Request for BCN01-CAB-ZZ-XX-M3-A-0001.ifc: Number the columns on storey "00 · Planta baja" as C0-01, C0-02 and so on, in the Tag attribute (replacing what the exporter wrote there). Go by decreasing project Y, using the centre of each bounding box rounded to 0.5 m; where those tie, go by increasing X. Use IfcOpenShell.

First a look at what the model holds.

```python
import ifcopenshell
import ifcopenshell.util.element
import ifcopenshell.util.placement

model = ifcopenshell.open("BCN01-CAB-ZZ-XX-M3-A-0001.ifc")
print(model.schema)
storey = next(s for s in model.by_type("IfcBuildingStorey") if s.Name == "00 · Planta baja")
columns = [e for e in ifcopenshell.util.element.get_decomposition(storey) if e.is_a("IfcColumn")]
for e in sorted(columns, key=lambda e: e.id()):
    origin = ifcopenshell.util.placement.get_local_placement(e.ObjectPlacement)[:3, 3]
    print(e.id(), e.Tag, e.Name, origin.round(2) + 0.0, sep=" | ")
```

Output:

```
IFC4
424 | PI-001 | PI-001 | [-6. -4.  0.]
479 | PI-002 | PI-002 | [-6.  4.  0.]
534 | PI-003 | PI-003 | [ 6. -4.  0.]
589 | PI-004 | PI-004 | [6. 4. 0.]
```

```python
import ifcopenshell
import ifcopenshell.geom
import ifcopenshell.util.element
import ifcopenshell.util.shape

model = ifcopenshell.open("BCN01-CAB-ZZ-XX-M3-A-0001.ifc")
settings = ifcopenshell.geom.settings()
settings.set("use-world-coords", True)


def centre(element):
    shape = ifcopenshell.geom.create_shape(settings, element)
    return ifcopenshell.util.shape.get_bbox_centroid(shape.geometry)


storey = next(s for s in model.by_type("IfcBuildingStorey") if s.Name == "00 · Planta baja")
columns = [e for e in ifcopenshell.util.element.get_decomposition(storey) if e.is_a("IfcColumn")]

# Insertion points can sit at a corner or the storey origin, so sort by the geometry (in metres).
centres = {e: centre(e) for e in columns}
columns.sort(key=lambda e: (-round(centres[e][1] / 0.5), centres[e][0]))

for i, e in enumerate(columns, start=1):
    number = f"C0-{i:02d}"
    e.Tag = number
    print(e.id(), number)

model.write("BCN01-CAB-ZZ-XX-M3-A-0001_rev.ifc")
```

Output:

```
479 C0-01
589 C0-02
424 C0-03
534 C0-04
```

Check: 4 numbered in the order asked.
